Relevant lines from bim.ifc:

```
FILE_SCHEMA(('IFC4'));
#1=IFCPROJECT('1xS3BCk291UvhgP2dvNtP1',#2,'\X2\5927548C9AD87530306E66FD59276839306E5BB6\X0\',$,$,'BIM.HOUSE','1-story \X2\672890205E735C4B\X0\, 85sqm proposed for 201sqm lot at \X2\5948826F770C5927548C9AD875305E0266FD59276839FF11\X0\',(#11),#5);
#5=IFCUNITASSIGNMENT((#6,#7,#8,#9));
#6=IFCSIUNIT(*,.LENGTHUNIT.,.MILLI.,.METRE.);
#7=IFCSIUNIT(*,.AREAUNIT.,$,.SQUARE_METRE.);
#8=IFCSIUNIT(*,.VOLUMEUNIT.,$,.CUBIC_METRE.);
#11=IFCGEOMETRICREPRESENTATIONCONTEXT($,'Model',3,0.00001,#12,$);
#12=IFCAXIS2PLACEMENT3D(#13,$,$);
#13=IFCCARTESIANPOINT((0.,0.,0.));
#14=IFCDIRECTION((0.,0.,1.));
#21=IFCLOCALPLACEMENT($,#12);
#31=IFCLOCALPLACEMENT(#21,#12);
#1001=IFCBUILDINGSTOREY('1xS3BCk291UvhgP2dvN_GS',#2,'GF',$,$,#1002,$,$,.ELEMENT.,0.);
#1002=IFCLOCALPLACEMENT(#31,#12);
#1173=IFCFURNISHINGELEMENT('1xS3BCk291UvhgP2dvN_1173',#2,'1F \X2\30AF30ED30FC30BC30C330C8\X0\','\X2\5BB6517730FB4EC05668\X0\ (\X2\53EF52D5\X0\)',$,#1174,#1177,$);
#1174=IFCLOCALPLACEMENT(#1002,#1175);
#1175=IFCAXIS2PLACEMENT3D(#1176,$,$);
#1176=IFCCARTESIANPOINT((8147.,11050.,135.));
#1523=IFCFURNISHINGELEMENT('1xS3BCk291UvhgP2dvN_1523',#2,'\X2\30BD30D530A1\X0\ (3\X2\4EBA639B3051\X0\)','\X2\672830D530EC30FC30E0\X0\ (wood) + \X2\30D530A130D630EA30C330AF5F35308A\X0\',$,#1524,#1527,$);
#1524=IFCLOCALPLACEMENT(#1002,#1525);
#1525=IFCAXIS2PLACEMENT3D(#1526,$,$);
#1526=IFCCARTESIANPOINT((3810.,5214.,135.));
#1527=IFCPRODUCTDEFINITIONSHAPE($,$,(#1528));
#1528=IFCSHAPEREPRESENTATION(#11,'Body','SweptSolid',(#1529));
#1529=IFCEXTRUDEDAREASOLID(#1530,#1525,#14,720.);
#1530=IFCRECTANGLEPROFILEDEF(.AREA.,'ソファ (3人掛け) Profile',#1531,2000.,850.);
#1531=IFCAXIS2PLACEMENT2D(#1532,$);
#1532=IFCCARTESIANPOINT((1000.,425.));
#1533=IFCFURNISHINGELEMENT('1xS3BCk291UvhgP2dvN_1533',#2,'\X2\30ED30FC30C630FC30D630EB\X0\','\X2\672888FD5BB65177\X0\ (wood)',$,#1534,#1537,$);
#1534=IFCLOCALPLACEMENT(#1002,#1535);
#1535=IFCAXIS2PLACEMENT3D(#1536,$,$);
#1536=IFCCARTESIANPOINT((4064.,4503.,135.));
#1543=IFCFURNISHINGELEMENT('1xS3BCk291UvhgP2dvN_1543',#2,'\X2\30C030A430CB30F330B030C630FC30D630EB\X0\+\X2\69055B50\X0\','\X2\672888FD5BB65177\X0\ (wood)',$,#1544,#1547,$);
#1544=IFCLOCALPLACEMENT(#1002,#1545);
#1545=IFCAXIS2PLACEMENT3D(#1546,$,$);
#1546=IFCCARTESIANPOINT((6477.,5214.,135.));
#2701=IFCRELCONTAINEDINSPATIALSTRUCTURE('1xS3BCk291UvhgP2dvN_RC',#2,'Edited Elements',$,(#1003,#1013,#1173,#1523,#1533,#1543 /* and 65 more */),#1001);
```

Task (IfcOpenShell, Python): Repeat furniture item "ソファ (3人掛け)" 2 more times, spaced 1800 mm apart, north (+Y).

```python
import numpy as np
import ifcopenshell
import ifcopenshell.api.geometry
import ifcopenshell.api.root
import ifcopenshell.util.element
import ifcopenshell.util.placement
import ifcopenshell.util.unit

model = ifcopenshell.open("bim.ifc")
unit_scale = ifcopenshell.util.unit.calculate_unit_scale(model)


def reuse_history(source, copy):
    """copy_class also copies each property set's owner history, people and application; keep the originals."""
    for rel in copy.IsDefinedBy:
        if rel.is_a("IfcRelDefinesByProperties") and (history := rel.RelatingPropertyDefinition.OwnerHistory):
            rel.RelatingPropertyDefinition.OwnerHistory = source.OwnerHistory
            ifcopenshell.util.element.remove_deep2(model, history)


source = model.by_guid("1xS3BCk291UvhgP2dvN_1523")
base = ifcopenshell.util.placement.get_local_placement(source.ObjectPlacement)
step = np.array([0.0, 1.0, 0.0]) * 1.8 / unit_scale

for i in range(1, 3):
    copy = ifcopenshell.api.root.copy_class(model, product=source)
    copy.Representation = ifcopenshell.util.element.copy_deep(
        model, source.Representation, exclude=["IfcGeometricRepresentationContext", "IfcRepresentationMap"]
    )
    reuse_history(source, copy)
    matrix = base.copy()
    matrix[:3, 3] += i * step
    print("added at", matrix[:3, 3].round(3) + 0.0)
    ifcopenshell.api.geometry.edit_object_placement(model, product=copy, matrix=matrix, is_si=False)

model.write("bim_rev.ifc")
```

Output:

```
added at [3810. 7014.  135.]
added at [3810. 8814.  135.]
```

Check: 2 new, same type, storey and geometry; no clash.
